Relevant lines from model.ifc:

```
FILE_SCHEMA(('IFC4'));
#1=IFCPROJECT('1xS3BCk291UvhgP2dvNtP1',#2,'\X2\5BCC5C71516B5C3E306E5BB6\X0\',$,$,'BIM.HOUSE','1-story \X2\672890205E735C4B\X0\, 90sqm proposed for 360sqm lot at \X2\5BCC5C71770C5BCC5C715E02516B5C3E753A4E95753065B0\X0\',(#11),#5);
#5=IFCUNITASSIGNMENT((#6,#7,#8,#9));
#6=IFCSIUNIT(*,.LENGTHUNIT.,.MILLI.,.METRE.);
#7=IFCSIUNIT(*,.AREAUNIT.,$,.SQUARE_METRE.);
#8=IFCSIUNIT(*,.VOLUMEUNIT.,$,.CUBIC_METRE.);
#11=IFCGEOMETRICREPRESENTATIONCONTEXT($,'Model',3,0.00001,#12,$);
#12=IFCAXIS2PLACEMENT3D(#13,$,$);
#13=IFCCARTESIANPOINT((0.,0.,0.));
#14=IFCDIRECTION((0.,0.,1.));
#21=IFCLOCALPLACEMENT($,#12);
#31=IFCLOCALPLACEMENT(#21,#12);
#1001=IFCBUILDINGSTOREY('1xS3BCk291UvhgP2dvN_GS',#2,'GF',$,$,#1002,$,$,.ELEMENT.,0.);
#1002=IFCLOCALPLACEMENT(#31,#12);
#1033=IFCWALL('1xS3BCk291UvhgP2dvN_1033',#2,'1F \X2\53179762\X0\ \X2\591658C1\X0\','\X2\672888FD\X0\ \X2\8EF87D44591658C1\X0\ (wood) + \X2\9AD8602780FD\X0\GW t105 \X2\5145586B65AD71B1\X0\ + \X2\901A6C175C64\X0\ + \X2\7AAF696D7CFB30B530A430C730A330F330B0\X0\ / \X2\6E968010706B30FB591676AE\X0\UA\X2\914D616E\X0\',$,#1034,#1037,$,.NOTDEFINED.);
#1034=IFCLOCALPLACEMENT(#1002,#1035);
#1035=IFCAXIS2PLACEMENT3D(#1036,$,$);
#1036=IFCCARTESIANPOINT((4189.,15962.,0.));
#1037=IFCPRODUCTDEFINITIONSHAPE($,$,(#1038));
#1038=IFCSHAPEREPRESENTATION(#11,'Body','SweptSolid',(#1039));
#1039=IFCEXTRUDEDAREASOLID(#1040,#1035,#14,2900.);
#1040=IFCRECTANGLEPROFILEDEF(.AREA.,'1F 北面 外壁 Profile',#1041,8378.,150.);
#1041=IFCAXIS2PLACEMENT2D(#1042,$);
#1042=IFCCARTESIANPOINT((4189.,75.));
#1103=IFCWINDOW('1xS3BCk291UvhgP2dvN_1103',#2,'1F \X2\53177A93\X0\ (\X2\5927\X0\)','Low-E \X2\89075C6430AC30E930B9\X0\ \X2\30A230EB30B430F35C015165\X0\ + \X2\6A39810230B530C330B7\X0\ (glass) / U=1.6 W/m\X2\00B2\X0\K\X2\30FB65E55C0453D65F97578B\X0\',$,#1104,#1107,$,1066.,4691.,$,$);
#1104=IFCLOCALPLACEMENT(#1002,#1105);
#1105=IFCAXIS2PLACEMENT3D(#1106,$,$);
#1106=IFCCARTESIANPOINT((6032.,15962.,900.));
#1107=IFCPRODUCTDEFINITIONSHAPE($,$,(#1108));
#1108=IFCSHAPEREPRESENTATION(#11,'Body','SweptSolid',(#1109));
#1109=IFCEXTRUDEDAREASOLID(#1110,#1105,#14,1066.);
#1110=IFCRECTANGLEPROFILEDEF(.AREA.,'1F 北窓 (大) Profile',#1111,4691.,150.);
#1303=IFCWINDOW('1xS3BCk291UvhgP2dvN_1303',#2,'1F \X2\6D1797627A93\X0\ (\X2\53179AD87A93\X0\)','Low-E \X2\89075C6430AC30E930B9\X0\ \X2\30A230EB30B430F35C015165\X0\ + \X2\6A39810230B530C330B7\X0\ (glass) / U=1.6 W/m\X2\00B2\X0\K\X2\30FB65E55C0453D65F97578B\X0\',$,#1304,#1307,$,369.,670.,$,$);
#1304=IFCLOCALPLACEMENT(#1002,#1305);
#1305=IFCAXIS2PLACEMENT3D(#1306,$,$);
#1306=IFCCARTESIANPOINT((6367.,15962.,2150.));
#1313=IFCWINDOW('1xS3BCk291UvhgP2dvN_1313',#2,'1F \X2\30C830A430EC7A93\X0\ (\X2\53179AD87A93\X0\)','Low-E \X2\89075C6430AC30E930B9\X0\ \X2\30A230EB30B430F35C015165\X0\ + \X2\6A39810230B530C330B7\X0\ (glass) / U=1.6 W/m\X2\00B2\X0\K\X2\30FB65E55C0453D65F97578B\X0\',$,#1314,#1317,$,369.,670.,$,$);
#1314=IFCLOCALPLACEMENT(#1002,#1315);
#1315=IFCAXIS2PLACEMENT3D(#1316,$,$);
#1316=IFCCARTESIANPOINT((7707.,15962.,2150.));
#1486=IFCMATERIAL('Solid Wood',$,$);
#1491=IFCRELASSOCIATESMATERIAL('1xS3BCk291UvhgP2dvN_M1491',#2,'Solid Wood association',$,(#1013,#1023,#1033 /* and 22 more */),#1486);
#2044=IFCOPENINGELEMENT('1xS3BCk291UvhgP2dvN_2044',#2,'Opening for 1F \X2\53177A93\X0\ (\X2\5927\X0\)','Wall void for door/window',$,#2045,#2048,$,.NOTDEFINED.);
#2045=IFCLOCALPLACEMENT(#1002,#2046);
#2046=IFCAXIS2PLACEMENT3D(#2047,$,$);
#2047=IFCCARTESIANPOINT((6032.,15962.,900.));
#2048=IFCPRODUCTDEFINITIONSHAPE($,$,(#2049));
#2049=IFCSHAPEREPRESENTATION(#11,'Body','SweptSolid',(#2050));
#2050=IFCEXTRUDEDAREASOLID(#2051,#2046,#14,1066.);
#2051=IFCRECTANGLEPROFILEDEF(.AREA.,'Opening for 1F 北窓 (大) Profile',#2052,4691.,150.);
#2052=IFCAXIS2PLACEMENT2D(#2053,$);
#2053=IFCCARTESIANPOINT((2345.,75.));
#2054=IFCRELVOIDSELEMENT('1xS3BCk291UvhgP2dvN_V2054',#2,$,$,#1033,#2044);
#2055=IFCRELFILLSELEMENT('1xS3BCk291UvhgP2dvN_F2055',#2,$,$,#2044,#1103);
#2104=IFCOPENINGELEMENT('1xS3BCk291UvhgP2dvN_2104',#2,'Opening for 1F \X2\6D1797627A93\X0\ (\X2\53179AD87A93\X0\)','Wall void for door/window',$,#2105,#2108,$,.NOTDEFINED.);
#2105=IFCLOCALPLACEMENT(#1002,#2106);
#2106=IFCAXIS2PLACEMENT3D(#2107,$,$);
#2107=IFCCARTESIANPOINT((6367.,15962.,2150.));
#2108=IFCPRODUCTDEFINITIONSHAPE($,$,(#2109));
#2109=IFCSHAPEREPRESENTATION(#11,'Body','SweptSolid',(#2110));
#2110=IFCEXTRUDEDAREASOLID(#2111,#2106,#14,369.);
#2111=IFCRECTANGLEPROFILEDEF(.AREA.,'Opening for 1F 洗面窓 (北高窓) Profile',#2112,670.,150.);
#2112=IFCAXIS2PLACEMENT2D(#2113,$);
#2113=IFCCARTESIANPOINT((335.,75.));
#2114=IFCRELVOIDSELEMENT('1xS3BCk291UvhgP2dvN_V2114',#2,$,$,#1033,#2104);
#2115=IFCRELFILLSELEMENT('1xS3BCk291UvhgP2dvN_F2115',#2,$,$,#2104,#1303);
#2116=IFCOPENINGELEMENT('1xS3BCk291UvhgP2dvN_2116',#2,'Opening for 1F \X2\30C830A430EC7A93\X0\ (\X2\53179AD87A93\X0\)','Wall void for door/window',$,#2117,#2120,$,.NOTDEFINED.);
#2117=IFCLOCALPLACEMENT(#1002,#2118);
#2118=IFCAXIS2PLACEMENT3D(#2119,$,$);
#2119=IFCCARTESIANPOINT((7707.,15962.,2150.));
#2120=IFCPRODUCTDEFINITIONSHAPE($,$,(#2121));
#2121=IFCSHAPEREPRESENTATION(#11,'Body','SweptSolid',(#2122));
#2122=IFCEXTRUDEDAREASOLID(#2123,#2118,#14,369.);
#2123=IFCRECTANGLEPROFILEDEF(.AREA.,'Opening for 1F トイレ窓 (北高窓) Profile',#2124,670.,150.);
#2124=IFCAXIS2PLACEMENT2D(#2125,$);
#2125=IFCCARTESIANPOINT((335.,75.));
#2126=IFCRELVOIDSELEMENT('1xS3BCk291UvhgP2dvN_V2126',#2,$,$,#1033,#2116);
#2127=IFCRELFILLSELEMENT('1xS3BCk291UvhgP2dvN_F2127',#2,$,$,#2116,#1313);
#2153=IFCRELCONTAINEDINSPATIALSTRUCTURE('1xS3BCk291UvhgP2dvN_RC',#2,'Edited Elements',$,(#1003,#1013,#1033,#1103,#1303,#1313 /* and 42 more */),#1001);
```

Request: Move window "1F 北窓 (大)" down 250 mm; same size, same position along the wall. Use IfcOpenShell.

```python
import numpy as np
import ifcopenshell
import ifcopenshell.api.geometry
import ifcopenshell.util.placement
import ifcopenshell.util.unit

model = ifcopenshell.open("model.ifc")
unit_scale = ifcopenshell.util.unit.calculate_unit_scale(model)

window = model.by_guid("1xS3BCk291UvhgP2dvN_1103")
opening = window.FillsVoids[0].RelatingOpeningElement
dz = -0.25 / unit_scale

shift = np.array([0.0, 0.0, dz])
# The window is not placed relative to its opening, so move both.
for product in (opening, window):
    matrix = ifcopenshell.util.placement.get_local_placement(product.ObjectPlacement)
    matrix[:3, 3] += shift
    ifcopenshell.api.geometry.edit_object_placement(model, product=product, matrix=matrix, is_si=False)

print(f"moved by {dz * unit_scale:+.3f} m")

model.write("model_rev.ifc")
```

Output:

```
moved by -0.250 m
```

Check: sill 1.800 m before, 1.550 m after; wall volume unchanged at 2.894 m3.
